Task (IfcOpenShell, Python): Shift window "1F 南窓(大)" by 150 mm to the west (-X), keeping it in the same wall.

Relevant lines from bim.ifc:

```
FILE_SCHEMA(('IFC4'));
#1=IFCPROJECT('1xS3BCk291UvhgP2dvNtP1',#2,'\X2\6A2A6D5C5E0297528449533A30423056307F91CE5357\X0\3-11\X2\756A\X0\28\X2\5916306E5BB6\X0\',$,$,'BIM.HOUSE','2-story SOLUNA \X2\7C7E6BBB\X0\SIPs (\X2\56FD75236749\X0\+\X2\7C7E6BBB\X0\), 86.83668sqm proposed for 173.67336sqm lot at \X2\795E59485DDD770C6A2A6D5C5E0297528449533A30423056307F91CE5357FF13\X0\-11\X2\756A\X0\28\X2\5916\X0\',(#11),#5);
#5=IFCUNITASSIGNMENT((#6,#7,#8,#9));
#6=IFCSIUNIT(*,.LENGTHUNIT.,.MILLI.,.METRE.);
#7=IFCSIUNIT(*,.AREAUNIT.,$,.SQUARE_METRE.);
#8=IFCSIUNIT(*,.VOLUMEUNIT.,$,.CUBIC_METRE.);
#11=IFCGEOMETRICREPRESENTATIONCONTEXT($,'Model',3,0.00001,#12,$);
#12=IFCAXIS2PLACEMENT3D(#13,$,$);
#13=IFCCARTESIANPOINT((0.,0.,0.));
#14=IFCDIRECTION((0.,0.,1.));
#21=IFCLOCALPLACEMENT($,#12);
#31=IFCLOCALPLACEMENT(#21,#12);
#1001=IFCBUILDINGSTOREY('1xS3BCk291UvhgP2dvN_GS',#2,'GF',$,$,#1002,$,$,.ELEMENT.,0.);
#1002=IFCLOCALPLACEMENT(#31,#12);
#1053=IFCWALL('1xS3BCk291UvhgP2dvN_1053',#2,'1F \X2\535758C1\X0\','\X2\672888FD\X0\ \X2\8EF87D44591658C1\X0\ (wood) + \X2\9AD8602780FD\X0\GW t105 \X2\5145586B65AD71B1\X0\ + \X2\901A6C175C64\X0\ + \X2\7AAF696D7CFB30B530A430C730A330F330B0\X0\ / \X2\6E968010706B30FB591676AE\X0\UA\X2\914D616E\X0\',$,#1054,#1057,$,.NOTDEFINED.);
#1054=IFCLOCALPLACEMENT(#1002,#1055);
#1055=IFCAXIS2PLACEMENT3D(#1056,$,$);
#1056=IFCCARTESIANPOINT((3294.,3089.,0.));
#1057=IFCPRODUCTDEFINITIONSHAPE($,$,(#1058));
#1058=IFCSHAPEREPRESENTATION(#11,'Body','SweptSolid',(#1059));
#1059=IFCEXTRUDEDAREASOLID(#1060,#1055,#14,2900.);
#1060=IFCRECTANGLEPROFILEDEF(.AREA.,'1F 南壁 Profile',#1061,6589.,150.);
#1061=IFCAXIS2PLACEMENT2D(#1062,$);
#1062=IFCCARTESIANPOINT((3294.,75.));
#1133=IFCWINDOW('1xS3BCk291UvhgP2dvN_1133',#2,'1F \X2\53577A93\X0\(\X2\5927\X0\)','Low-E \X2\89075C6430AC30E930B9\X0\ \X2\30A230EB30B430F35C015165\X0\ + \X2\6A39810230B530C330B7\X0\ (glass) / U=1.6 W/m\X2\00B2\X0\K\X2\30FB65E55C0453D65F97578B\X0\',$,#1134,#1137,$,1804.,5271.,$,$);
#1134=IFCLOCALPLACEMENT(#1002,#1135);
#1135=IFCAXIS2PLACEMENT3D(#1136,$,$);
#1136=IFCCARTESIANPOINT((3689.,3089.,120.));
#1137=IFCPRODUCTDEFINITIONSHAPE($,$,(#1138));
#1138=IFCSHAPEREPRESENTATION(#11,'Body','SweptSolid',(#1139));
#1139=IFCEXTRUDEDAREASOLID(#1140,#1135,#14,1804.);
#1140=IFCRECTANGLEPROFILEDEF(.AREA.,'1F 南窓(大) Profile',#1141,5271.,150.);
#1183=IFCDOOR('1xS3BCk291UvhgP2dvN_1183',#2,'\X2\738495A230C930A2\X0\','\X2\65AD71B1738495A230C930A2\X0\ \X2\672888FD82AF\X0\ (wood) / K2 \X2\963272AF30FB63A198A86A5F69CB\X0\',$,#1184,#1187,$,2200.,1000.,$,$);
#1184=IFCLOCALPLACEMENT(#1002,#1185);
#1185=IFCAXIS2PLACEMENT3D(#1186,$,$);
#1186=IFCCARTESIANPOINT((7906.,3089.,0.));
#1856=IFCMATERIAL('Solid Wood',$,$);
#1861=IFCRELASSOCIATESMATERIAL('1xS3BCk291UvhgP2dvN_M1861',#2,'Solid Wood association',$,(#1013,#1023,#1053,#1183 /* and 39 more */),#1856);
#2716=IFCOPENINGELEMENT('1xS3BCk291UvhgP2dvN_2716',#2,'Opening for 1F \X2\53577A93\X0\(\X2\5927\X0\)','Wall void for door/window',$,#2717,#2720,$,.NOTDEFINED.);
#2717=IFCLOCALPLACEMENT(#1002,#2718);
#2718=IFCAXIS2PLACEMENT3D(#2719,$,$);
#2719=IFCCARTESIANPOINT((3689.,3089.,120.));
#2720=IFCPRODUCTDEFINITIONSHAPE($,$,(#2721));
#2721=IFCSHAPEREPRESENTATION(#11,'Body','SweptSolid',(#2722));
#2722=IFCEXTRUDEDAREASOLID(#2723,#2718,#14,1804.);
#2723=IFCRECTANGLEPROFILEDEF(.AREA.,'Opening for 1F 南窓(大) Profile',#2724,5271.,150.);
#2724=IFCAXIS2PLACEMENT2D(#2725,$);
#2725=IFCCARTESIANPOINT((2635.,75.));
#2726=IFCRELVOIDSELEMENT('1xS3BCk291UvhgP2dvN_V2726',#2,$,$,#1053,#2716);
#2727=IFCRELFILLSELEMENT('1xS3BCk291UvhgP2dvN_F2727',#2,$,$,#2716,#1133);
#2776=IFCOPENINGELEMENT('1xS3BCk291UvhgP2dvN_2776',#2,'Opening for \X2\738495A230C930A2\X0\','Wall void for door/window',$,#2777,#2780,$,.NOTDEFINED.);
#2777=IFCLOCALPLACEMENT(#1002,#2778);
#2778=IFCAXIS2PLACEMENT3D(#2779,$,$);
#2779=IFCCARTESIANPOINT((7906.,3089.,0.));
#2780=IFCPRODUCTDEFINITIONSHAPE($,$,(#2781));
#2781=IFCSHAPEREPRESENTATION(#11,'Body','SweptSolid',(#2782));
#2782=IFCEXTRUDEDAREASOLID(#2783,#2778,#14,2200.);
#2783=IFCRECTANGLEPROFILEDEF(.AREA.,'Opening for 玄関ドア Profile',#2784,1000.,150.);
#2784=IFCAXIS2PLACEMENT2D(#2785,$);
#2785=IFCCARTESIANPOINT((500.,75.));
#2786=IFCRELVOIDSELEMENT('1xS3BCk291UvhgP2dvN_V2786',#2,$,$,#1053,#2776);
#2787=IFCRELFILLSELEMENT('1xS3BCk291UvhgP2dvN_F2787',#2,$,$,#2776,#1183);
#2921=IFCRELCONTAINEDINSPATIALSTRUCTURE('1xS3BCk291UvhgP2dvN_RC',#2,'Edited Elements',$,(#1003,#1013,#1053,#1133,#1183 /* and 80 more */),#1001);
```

```python
import ifcopenshell
import ifcopenshell.api.geometry
import ifcopenshell.util.placement
import ifcopenshell.util.unit

model = ifcopenshell.open("bim.ifc")
unit_scale = ifcopenshell.util.unit.calculate_unit_scale(model)

window = model.by_guid("1xS3BCk291UvhgP2dvN_1133")
opening = window.FillsVoids[0].RelatingOpeningElement
wall = opening.VoidsElements[0].RelatingBuildingElement

wall_matrix = ifcopenshell.util.placement.get_local_placement(wall.ObjectPlacement)
shift = wall_matrix[:3, 0] * -0.15 / unit_scale
before = ifcopenshell.util.placement.get_local_placement(window.ObjectPlacement)[:3, 3].copy()

# The window is not placed relative to its opening, so move both.
for product in (opening, window):
    matrix = ifcopenshell.util.placement.get_local_placement(product.ObjectPlacement)
    matrix[:3, 3] += shift
    ifcopenshell.api.geometry.edit_object_placement(model, product=product, matrix=matrix, is_si=False)

after = ifcopenshell.util.placement.get_local_placement(window.ObjectPlacement)[:3, 3]
print("window moved by", (after - before).round(3) + 0.0)

model.write("bim_updated.ifc")
```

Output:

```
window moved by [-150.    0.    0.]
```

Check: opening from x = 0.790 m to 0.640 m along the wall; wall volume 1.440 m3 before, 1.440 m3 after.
